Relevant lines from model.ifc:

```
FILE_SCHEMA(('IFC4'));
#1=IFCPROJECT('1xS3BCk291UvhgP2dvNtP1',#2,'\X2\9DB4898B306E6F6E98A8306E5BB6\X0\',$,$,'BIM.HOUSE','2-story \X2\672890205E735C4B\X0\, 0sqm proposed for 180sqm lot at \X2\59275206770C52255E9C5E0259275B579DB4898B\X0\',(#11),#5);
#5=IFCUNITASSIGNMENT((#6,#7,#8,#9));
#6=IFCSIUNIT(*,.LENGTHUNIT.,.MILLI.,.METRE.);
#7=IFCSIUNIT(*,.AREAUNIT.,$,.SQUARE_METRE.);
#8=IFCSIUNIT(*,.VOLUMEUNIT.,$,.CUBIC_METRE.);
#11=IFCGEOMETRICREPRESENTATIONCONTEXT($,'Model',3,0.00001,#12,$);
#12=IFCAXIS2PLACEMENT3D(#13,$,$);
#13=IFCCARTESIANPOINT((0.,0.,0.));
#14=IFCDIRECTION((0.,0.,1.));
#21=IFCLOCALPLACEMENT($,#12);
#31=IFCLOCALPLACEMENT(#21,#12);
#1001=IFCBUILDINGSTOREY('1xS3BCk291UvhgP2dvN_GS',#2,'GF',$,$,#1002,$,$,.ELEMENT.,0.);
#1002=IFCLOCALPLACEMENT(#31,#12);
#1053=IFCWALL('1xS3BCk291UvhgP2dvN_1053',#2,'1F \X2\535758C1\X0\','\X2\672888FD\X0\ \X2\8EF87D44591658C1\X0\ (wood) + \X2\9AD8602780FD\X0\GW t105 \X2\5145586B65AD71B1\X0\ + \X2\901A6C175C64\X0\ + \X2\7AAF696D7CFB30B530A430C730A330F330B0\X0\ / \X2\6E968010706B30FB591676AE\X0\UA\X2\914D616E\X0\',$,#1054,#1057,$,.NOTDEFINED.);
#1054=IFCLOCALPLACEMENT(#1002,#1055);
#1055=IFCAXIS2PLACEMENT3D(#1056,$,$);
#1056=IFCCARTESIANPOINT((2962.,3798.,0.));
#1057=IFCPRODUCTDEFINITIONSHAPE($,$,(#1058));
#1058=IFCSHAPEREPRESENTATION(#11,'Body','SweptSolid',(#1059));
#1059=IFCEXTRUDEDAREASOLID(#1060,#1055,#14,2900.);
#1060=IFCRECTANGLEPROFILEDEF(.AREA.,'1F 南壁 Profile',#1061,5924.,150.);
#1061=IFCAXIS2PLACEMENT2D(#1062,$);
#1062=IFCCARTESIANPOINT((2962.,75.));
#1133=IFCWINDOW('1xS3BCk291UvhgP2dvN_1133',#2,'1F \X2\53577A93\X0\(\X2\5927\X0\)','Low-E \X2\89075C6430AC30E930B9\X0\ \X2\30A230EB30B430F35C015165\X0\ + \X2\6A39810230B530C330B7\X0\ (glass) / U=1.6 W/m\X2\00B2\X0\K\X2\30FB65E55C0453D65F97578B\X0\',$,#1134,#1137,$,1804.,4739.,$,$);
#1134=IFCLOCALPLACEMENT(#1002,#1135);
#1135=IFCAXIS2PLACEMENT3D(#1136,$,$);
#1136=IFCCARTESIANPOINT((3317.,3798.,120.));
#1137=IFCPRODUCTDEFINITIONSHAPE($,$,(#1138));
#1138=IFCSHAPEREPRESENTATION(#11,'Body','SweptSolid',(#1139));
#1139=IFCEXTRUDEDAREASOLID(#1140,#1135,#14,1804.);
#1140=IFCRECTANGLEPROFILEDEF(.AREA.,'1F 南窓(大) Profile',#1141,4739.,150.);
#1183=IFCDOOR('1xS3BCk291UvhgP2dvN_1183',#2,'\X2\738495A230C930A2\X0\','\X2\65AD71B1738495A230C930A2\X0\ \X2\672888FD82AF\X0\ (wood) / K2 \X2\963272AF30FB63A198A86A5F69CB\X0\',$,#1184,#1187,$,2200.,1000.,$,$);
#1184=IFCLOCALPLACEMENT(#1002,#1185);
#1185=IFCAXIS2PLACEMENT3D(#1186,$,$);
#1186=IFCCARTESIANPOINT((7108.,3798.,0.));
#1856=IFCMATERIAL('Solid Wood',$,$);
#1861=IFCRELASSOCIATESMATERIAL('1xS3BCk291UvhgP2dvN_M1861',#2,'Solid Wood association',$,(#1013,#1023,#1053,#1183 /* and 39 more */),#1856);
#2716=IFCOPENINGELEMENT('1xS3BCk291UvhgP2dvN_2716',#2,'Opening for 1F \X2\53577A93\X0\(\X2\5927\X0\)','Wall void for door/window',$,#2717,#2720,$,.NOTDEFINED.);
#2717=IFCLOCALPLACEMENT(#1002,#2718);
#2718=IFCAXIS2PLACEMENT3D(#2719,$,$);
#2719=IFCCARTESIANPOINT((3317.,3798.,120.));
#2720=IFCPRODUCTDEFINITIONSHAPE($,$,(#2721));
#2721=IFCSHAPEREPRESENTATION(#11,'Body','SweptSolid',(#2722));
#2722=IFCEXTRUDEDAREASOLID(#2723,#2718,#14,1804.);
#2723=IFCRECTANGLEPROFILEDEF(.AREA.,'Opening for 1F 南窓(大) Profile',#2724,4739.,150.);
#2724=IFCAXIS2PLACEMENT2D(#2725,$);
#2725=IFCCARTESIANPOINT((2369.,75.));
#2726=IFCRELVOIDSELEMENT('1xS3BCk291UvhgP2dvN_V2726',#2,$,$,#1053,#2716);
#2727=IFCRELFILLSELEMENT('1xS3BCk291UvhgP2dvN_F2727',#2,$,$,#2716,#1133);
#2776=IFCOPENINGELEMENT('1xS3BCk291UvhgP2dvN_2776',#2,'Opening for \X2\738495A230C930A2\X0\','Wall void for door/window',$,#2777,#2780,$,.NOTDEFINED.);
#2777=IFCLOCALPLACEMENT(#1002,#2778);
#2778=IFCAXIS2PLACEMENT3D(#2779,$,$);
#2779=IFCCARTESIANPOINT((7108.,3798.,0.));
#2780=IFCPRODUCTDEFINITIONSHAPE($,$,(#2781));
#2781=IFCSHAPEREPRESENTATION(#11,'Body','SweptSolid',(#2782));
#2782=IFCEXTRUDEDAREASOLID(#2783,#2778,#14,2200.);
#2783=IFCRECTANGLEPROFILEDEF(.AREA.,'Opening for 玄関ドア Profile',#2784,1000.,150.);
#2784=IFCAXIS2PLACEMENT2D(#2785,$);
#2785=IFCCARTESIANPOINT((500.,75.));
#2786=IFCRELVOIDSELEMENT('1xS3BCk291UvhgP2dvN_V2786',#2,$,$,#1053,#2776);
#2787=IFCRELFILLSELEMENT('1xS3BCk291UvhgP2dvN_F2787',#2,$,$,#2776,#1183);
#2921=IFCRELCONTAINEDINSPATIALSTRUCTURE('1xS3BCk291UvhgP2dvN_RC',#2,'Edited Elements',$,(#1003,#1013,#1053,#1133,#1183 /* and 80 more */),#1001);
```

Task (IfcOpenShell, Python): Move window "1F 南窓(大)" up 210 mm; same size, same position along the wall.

```python
import numpy as np
import ifcopenshell
import ifcopenshell.api.geometry
import ifcopenshell.util.placement
import ifcopenshell.util.unit

model = ifcopenshell.open("model.ifc")
unit_scale = ifcopenshell.util.unit.calculate_unit_scale(model)

window = model.by_guid("1xS3BCk291UvhgP2dvN_1133")
opening = window.FillsVoids[0].RelatingOpeningElement
dz = 210.0

shift = np.array([0.0, 0.0, dz])
# The window is not placed relative to its opening, so move both.
for product in (opening, window):
    matrix = ifcopenshell.util.placement.get_local_placement(product.ObjectPlacement)
    matrix[:3, 3] += shift
    ifcopenshell.api.geometry.edit_object_placement(model, product=product, matrix=matrix, is_si=False)

print(f"moved by {dz * unit_scale:+.3f} m")

model.write("model_rev.ifc")
```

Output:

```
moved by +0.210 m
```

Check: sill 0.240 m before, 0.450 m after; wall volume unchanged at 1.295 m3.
